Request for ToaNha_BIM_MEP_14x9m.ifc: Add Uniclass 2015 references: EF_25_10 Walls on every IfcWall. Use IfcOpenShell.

First a look at what the model holds.

```python
import ifcopenshell

model = ifcopenshell.open("ToaNha_BIM_MEP_14x9m.ifc")
print(model.schema)
print("classifications:", [c.Name for c in model.by_type("IfcClassification")])
for ifc_class in ("IfcDoor", "IfcRoof", "IfcStair", "IfcWall", "IfcWindow"):
    print(ifc_class, len(model.by_type(ifc_class)))
```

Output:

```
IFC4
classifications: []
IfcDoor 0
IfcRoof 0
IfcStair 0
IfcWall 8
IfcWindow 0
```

```python
import ifcopenshell
import ifcopenshell.api.classification

model = ifcopenshell.open("ToaNha_BIM_MEP_14x9m.ifc")

system = ifcopenshell.api.classification.add_classification(model, classification="Uniclass 2015")

codes = {
    "IfcWall": ("EF_25_10", "Walls"),
}
for ifc_class, (code, name) in codes.items():
    products = model.by_type(ifc_class)
    ifcopenshell.api.classification.add_reference(
        model, products=products, classification=system, identification=code, name=name
    )
    print(code, len(products))

model.write("ToaNha_BIM_MEP_14x9m-out.ifc")
```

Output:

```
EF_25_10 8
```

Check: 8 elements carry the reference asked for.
